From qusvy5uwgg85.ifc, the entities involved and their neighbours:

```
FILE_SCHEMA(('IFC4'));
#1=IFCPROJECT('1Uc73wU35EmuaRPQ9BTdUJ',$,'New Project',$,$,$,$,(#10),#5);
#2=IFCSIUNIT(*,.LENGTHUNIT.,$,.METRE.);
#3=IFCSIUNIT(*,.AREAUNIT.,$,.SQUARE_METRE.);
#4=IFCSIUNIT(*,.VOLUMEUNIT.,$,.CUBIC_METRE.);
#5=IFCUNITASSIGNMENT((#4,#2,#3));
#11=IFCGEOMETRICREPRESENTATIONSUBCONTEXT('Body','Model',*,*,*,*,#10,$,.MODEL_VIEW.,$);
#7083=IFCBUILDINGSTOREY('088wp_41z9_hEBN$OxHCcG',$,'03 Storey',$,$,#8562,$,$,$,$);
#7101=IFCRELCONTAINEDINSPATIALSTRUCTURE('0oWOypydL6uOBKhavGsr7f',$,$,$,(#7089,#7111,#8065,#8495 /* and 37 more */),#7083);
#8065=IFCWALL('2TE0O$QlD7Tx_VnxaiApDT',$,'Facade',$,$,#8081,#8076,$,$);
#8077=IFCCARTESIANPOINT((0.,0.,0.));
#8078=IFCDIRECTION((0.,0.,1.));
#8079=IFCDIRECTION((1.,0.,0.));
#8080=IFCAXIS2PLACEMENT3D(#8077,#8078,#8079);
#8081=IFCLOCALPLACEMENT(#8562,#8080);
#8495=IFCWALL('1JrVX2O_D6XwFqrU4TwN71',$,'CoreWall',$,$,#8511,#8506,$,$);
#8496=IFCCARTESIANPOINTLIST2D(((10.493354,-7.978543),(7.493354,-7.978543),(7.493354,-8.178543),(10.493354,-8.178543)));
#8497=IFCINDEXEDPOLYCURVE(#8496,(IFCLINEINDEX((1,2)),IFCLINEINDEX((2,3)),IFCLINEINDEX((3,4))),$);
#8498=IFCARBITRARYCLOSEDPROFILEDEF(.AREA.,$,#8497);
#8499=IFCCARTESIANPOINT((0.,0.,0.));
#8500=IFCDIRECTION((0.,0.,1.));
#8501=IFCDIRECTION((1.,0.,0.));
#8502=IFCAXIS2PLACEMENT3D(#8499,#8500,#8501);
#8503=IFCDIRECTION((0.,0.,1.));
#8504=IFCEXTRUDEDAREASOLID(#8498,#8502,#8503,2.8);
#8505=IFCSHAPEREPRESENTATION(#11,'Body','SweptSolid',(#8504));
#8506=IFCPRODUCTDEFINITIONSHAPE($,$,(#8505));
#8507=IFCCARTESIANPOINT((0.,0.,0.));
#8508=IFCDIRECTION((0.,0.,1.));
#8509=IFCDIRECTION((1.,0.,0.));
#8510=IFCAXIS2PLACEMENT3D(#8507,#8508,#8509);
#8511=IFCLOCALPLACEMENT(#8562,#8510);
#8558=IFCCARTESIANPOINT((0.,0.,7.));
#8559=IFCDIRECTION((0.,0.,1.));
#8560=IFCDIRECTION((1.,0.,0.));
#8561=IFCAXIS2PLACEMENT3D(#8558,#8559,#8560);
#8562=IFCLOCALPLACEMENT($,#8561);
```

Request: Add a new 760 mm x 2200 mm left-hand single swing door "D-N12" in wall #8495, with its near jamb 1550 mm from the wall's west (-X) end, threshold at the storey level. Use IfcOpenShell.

```python
import numpy as np
import ifcopenshell
import ifcopenshell.api.feature
import ifcopenshell.api.geometry
import ifcopenshell.api.root
import ifcopenshell.api.spatial
import ifcopenshell.geom
import ifcopenshell.util.element
import ifcopenshell.util.placement
import ifcopenshell.util.representation
import ifcopenshell.util.shape
import ifcopenshell.util.unit

model = ifcopenshell.open("qusvy5uwgg85.ifc")
unit_scale = ifcopenshell.util.unit.calculate_unit_scale(model)
settings = ifcopenshell.geom.settings()


def volume(element):
    """Net volume in cubic metres, openings subtracted."""
    shape = ifcopenshell.geom.create_shape(settings, element)
    return ifcopenshell.util.shape.get_volume(shape.geometry)


wall = model.by_id(8495)
storey = ifcopenshell.util.element.get_container(wall, ifc_class="IfcBuildingStorey")
context = ifcopenshell.util.representation.get_context(model, "Model", "Body", "MODEL_VIEW")
before = volume(wall)

width, height, from_end, sill = 0.76, 2.2, 1.55, 0.0  # metres

# The wall runs along its own X axis, and the end named is its -X end.
wall_shape = ifcopenshell.geom.create_shape(settings, wall)
x, y, z = ifcopenshell.util.shape.get_vertices(wall_shape.geometry).T
start = x.min() + from_end
face, thickness = float(y.min()), float(y.max() - y.min())
wall_matrix = ifcopenshell.util.placement.get_local_placement(wall.ObjectPlacement)
level = ifcopenshell.util.placement.get_local_placement(storey.ObjectPlacement)[2, 3]


def in_wall(x, y):
    """Placement at x, y metres in the wall's axes, at sill height."""
    matrix = wall_matrix.copy()
    matrix[:, 3] = wall_matrix @ np.array([x / unit_scale, y / unit_scale, 0.0, 1.0])
    matrix[2, 3] = level + sill / unit_scale
    return matrix


# Opening: a box that overshoots both wall faces by 50 mm.
opening = ifcopenshell.api.root.create_entity(model, ifc_class="IfcOpeningElement", predefined_type="OPENING")
box = ifcopenshell.api.geometry.add_wall_representation(
    model, context=context, length=width, height=height, thickness=thickness + 0.1
)
ifcopenshell.api.geometry.assign_representation(model, product=opening, representation=box)
ifcopenshell.api.geometry.edit_object_placement(model, product=opening, matrix=in_wall(start, face - 0.05), is_si=False)
ifcopenshell.api.feature.add_feature(model, feature=opening, element=wall)

door = ifcopenshell.api.root.create_entity(model, ifc_class="IfcDoor", name="D-N12", predefined_type="DOOR")
door.OverallWidth, door.OverallHeight = width / unit_scale, height / unit_scale
door.OperationType = "SINGLE_SWING_LEFT"
body = ifcopenshell.api.geometry.add_door_representation(
    model,
    context=context,
    overall_width=door.OverallWidth,
    overall_height=door.OverallHeight,
    operation_type="SINGLE_SWING_LEFT",
    lining_properties={"LiningDepth": thickness / unit_scale, "ThresholdDepth": thickness / unit_scale},
)
ifcopenshell.api.geometry.assign_representation(model, product=door, representation=body)
ifcopenshell.api.spatial.assign_container(model, products=[door], relating_structure=storey)
ifcopenshell.api.feature.add_filling(model, opening=opening, element=door)

# The lining spans the wall, so the door starts at the wall face.
ifcopenshell.api.geometry.edit_object_placement(model, product=door, matrix=in_wall(start, face), is_si=False)

after = volume(wall)

print(f"wall volume {before:.3f} -> {after:.3f} m3")

model.write("qusvy5uwgg85_edited.ifc")
```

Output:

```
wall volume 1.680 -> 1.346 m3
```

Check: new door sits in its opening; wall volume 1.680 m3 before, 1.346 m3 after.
